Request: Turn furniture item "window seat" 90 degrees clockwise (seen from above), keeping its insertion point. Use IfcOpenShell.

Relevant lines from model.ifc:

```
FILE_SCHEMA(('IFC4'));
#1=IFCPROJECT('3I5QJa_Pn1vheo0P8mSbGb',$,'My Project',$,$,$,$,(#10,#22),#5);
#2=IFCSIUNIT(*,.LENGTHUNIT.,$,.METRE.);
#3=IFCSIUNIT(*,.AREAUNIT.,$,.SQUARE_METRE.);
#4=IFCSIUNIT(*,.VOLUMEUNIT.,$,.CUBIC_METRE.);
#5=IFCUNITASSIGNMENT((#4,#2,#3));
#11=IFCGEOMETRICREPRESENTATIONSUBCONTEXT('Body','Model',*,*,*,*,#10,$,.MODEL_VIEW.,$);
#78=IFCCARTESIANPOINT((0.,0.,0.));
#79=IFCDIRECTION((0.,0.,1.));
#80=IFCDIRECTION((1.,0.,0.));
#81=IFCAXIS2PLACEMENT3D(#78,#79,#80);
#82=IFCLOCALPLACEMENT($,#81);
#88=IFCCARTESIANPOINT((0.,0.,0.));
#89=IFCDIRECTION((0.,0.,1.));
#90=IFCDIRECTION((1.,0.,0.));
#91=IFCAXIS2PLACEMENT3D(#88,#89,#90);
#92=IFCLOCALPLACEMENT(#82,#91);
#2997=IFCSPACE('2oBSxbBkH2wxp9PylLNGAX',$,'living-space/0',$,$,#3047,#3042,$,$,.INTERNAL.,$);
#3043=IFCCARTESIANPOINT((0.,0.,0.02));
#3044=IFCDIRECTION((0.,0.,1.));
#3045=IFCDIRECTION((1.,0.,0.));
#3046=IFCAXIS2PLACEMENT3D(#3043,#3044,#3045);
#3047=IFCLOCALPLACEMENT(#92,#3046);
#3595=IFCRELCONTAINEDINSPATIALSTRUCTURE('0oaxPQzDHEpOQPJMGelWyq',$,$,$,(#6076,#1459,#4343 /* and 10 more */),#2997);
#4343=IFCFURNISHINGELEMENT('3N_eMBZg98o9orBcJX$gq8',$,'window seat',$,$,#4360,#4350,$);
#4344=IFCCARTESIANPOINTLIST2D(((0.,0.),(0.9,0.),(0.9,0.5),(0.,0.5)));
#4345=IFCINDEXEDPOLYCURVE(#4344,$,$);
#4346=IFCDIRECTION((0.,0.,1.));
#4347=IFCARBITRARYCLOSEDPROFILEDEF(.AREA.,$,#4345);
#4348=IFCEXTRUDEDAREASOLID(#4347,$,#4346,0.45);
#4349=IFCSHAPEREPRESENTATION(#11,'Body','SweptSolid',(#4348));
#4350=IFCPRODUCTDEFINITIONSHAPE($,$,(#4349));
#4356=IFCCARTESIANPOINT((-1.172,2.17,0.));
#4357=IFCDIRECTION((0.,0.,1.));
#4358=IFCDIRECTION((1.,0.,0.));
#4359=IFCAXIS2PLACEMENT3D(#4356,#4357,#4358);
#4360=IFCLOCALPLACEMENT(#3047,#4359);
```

```python
import ifcopenshell
import ifcopenshell.api.geometry
import ifcopenshell.util.placement

model = ifcopenshell.open("model.ifc")

item = model.by_id(4343)
matrix = ifcopenshell.util.placement.get_local_placement(item.ObjectPlacement)
matrix = matrix @ ifcopenshell.util.placement.rotation(-90, "Z")
ifcopenshell.api.geometry.edit_object_placement(model, product=item, matrix=matrix, is_si=False)

print(ifcopenshell.util.placement.get_local_placement(item.ObjectPlacement).round(3) + 0.0)

model.write("model_v2.ifc")
```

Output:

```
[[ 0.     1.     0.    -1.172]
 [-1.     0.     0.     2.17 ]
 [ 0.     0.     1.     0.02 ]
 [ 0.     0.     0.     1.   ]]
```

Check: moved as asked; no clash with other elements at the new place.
